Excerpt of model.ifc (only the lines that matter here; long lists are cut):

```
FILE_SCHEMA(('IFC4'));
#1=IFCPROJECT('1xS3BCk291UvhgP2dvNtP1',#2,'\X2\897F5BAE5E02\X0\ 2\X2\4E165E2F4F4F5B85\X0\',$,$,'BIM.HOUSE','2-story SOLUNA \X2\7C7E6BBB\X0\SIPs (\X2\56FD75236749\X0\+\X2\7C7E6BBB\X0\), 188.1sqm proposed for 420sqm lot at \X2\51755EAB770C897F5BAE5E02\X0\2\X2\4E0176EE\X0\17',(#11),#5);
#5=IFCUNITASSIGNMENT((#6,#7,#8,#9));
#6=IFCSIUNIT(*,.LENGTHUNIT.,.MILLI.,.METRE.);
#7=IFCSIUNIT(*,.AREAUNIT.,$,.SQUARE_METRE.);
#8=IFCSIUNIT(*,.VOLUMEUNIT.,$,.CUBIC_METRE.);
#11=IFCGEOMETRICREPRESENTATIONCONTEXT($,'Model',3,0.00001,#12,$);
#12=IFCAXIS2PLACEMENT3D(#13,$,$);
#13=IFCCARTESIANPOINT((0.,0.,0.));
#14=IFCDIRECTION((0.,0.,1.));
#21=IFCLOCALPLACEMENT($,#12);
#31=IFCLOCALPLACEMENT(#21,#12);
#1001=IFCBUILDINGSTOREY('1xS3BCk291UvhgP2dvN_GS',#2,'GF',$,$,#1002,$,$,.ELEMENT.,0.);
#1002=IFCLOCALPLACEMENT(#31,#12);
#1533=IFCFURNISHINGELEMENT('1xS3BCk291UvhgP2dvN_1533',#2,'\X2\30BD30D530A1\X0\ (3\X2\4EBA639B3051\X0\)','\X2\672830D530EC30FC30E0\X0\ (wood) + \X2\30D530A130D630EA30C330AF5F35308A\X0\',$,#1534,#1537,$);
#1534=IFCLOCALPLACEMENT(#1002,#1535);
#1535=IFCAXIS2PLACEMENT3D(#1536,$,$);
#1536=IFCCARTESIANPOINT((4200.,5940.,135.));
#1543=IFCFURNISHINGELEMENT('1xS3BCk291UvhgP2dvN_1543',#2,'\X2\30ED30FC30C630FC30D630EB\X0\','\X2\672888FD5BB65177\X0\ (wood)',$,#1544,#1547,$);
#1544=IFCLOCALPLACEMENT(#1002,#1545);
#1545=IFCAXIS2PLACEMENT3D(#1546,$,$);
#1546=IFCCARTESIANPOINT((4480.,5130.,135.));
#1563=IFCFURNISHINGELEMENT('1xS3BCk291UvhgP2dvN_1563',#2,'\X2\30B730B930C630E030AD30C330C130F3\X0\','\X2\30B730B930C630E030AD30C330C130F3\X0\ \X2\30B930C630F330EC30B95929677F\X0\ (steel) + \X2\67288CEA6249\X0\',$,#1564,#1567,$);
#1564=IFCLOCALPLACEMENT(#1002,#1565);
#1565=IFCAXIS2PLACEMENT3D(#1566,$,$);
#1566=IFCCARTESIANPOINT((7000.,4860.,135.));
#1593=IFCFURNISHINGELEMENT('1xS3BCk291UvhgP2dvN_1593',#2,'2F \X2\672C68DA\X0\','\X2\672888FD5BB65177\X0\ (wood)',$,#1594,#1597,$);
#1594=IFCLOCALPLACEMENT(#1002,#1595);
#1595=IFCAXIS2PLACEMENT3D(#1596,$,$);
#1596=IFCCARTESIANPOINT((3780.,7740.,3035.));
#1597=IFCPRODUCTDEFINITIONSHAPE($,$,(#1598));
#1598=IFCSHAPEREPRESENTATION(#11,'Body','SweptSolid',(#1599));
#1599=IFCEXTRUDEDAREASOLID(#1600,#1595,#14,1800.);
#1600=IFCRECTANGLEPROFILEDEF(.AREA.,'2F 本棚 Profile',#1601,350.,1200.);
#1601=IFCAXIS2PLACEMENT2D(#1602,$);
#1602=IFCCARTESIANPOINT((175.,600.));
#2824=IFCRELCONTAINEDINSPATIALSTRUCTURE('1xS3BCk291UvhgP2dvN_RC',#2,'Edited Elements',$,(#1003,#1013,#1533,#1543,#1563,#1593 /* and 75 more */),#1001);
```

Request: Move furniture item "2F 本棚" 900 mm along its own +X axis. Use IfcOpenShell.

```python
import ifcopenshell
import ifcopenshell.api.geometry
import ifcopenshell.util.placement

model = ifcopenshell.open("model.ifc")

item = model.by_id(1593)
matrix = ifcopenshell.util.placement.get_local_placement(item.ObjectPlacement)
matrix[:3, 3] += matrix[:3, 0] * 900.0
ifcopenshell.api.geometry.edit_object_placement(model, product=item, matrix=matrix, is_si=False)

print(ifcopenshell.util.placement.get_local_placement(item.ObjectPlacement).round(3) + 0.0)

model.write("model_updated.ifc")
```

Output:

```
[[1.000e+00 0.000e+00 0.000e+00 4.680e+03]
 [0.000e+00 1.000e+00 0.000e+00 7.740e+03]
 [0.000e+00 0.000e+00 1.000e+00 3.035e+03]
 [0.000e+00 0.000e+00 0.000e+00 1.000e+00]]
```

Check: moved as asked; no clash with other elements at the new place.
